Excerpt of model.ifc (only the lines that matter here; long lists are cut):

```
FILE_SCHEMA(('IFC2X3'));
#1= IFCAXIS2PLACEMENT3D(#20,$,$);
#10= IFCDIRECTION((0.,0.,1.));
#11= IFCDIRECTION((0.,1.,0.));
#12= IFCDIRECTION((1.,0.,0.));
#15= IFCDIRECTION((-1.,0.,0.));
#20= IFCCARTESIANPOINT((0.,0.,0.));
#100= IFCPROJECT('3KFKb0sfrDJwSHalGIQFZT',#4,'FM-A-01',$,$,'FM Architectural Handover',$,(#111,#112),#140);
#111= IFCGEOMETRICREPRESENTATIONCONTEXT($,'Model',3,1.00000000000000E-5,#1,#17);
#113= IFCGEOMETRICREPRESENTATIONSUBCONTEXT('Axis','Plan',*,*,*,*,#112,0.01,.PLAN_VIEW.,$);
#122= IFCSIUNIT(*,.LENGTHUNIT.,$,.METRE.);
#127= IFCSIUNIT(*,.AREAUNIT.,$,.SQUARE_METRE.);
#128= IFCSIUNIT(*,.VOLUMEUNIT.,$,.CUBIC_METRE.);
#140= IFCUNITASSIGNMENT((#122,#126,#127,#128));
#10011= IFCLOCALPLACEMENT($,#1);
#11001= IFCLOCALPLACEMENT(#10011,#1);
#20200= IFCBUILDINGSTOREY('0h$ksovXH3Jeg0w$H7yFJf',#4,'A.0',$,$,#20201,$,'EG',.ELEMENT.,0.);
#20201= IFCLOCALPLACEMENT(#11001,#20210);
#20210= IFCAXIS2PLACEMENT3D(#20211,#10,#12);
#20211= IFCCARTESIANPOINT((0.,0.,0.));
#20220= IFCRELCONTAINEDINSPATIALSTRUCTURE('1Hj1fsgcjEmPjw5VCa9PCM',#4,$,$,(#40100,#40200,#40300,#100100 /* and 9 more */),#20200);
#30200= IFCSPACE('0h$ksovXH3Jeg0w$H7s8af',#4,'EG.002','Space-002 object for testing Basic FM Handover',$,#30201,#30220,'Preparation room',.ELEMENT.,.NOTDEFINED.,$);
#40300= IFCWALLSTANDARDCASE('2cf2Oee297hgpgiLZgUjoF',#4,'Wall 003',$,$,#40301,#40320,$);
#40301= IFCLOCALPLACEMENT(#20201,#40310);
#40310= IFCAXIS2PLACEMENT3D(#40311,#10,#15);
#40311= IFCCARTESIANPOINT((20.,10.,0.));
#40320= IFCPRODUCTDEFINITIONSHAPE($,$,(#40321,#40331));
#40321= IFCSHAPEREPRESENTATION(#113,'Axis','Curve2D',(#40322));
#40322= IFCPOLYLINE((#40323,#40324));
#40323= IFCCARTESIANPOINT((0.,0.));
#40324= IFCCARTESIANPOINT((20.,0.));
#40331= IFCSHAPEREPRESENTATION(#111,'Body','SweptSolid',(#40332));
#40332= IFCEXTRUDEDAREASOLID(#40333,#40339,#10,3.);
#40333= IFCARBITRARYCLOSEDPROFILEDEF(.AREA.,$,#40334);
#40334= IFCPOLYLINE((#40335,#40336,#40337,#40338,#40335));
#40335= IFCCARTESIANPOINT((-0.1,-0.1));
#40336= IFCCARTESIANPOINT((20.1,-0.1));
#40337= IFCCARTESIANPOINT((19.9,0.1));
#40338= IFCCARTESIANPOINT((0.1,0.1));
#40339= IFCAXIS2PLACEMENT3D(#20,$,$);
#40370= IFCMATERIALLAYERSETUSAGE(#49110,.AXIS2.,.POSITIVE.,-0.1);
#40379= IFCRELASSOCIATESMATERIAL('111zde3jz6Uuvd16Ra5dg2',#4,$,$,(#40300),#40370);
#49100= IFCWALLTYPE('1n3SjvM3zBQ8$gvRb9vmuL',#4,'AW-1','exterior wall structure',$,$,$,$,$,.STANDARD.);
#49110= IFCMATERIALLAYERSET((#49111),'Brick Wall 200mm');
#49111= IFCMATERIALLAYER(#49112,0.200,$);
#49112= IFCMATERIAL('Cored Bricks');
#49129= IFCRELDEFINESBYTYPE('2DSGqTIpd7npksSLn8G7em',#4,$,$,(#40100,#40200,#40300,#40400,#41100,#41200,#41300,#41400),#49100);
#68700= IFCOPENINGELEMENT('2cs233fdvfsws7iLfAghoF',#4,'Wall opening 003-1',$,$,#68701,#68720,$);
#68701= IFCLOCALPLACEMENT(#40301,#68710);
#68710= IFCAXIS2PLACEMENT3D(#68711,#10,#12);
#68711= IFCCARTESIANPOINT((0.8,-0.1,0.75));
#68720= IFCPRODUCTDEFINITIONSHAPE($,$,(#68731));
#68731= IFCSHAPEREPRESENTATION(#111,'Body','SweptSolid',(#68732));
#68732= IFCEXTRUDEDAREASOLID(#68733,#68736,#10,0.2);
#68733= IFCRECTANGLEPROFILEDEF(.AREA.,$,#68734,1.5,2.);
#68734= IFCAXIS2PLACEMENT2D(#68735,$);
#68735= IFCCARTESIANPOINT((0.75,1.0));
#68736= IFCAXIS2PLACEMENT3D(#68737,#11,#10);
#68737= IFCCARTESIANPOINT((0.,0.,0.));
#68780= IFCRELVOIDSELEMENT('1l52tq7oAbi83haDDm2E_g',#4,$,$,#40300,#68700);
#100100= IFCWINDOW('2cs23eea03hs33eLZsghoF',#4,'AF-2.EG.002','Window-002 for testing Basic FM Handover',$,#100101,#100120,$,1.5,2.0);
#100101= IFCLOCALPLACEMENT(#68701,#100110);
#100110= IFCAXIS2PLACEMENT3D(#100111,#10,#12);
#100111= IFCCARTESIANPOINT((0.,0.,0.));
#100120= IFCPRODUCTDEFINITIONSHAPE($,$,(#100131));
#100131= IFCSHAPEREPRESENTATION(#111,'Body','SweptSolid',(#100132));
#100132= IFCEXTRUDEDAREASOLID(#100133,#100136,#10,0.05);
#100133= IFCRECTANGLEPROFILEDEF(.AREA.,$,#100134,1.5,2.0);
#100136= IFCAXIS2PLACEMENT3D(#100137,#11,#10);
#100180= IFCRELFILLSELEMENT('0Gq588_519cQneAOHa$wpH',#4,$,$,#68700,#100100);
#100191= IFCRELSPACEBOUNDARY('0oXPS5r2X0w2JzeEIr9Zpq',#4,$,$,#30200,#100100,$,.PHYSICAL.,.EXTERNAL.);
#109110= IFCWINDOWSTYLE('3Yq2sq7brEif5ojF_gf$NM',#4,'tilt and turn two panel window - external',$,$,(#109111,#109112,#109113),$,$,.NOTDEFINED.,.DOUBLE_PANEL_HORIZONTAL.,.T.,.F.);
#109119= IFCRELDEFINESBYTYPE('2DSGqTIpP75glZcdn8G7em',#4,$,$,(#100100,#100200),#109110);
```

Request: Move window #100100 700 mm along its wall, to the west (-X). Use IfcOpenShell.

```python
import ifcopenshell
import ifcopenshell.api.geometry
import ifcopenshell.util.placement
import ifcopenshell.util.unit

model = ifcopenshell.open("model.ifc")
unit_scale = ifcopenshell.util.unit.calculate_unit_scale(model)

window = model.by_guid("2cs23eea03hs33eLZsghoF")
opening = window.FillsVoids[0].RelatingOpeningElement
wall = opening.VoidsElements[0].RelatingBuildingElement

wall_matrix = ifcopenshell.util.placement.get_local_placement(wall.ObjectPlacement)
shift = wall_matrix[:3, 0] * 0.7 / unit_scale
before = ifcopenshell.util.placement.get_local_placement(window.ObjectPlacement)[:3, 3].copy()

# The window is placed relative to its opening, so it follows when the opening moves.
matrix = ifcopenshell.util.placement.get_local_placement(opening.ObjectPlacement)
matrix[:3, 3] += shift
ifcopenshell.api.geometry.edit_object_placement(
    model, product=opening, matrix=matrix, is_si=False, should_transform_children=True
)

after = ifcopenshell.util.placement.get_local_placement(window.ObjectPlacement)[:3, 3]
print("window moved by", (after - before).round(3) + 0.0)

model.write("model_rev.ifc")
```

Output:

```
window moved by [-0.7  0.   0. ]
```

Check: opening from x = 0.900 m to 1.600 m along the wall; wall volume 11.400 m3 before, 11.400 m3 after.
